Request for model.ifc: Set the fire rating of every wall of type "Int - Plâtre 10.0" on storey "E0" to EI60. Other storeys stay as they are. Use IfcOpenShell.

First a look at what the model holds.

```python
import ifcopenshell
import ifcopenshell.util.element

model = ifcopenshell.open("model.ifc")
print(model.schema)
storey = next(s for s in model.by_type("IfcBuildingStorey") if s.Name == "E0")
walls = [e for e in ifcopenshell.util.element.get_decomposition(storey) if e.is_a("IfcWall")]
seen = {}
for e in walls:
    element_type = ifcopenshell.util.element.get_type(e)
    key = (element_type.Name if element_type != e and element_type else None, ifcopenshell.util.element.get_pset(e, "Pset_WallCommon", "FireRating"))
    seen[key] = seen.get(key, 0) + 1
for (name, value), count in sorted(seen.items(), key=str):
    print(count, "x", name, "|", value)
```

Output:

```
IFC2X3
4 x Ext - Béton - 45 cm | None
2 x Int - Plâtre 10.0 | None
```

```python
import ifcopenshell
import ifcopenshell.api.pset
import ifcopenshell.util.element

model = ifcopenshell.open("model.ifc")

storey = next(s for s in model.by_type("IfcBuildingStorey") if s.Name == "E0")
walls = [e for e in ifcopenshell.util.element.get_decomposition(storey) if e.is_a("IfcWall")]

count = 0
for e in walls:
    element_type = ifcopenshell.util.element.get_type(e)
    if element_type in (None, e) or element_type.Name != "Int - Plâtre 10.0":
        continue
    # add_pset returns the element's existing set when there is one.
    pset = ifcopenshell.api.pset.add_pset(model, product=e, name="Pset_WallCommon")
    ifcopenshell.api.pset.edit_pset(model, pset=pset, properties={"FireRating": "EI60"})
    count += 1

print(count, "walls updated")

model.write("model_edited.ifc")
```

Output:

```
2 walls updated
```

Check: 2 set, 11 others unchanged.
